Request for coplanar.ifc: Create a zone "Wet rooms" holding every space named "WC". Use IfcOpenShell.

First a look at what the model holds.

```python
import ifcopenshell

model = ifcopenshell.open("coplanar.ifc")
print(model.schema)
seen = {}
for space in model.by_type("IfcSpace"):
    seen[space.LongName] = seen.get(space.LongName, 0) + 1
for name, count in sorted(seen.items(), key=str):
    print(count, "x", name)
print("zones:", [z.Name for z in model.by_type("IfcZone")][:20])
```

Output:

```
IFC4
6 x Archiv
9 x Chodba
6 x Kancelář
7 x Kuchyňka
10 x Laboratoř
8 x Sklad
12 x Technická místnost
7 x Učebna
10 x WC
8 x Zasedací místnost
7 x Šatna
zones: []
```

```python
import ifcopenshell
import ifcopenshell.api.group
import ifcopenshell.api.root

model = ifcopenshell.open("coplanar.ifc")

names = {"WC"}
spaces = [s for s in model.by_type("IfcSpace") if s.LongName in names]

zone = ifcopenshell.api.root.create_entity(model, ifc_class="IfcZone", name="Wet rooms")
ifcopenshell.api.group.assign_group(model, products=spaces, group=zone)
print(len(spaces), "spaces in", zone.Name)

model.write("coplanar-out.ifc")
```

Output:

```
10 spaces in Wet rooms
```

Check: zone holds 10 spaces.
